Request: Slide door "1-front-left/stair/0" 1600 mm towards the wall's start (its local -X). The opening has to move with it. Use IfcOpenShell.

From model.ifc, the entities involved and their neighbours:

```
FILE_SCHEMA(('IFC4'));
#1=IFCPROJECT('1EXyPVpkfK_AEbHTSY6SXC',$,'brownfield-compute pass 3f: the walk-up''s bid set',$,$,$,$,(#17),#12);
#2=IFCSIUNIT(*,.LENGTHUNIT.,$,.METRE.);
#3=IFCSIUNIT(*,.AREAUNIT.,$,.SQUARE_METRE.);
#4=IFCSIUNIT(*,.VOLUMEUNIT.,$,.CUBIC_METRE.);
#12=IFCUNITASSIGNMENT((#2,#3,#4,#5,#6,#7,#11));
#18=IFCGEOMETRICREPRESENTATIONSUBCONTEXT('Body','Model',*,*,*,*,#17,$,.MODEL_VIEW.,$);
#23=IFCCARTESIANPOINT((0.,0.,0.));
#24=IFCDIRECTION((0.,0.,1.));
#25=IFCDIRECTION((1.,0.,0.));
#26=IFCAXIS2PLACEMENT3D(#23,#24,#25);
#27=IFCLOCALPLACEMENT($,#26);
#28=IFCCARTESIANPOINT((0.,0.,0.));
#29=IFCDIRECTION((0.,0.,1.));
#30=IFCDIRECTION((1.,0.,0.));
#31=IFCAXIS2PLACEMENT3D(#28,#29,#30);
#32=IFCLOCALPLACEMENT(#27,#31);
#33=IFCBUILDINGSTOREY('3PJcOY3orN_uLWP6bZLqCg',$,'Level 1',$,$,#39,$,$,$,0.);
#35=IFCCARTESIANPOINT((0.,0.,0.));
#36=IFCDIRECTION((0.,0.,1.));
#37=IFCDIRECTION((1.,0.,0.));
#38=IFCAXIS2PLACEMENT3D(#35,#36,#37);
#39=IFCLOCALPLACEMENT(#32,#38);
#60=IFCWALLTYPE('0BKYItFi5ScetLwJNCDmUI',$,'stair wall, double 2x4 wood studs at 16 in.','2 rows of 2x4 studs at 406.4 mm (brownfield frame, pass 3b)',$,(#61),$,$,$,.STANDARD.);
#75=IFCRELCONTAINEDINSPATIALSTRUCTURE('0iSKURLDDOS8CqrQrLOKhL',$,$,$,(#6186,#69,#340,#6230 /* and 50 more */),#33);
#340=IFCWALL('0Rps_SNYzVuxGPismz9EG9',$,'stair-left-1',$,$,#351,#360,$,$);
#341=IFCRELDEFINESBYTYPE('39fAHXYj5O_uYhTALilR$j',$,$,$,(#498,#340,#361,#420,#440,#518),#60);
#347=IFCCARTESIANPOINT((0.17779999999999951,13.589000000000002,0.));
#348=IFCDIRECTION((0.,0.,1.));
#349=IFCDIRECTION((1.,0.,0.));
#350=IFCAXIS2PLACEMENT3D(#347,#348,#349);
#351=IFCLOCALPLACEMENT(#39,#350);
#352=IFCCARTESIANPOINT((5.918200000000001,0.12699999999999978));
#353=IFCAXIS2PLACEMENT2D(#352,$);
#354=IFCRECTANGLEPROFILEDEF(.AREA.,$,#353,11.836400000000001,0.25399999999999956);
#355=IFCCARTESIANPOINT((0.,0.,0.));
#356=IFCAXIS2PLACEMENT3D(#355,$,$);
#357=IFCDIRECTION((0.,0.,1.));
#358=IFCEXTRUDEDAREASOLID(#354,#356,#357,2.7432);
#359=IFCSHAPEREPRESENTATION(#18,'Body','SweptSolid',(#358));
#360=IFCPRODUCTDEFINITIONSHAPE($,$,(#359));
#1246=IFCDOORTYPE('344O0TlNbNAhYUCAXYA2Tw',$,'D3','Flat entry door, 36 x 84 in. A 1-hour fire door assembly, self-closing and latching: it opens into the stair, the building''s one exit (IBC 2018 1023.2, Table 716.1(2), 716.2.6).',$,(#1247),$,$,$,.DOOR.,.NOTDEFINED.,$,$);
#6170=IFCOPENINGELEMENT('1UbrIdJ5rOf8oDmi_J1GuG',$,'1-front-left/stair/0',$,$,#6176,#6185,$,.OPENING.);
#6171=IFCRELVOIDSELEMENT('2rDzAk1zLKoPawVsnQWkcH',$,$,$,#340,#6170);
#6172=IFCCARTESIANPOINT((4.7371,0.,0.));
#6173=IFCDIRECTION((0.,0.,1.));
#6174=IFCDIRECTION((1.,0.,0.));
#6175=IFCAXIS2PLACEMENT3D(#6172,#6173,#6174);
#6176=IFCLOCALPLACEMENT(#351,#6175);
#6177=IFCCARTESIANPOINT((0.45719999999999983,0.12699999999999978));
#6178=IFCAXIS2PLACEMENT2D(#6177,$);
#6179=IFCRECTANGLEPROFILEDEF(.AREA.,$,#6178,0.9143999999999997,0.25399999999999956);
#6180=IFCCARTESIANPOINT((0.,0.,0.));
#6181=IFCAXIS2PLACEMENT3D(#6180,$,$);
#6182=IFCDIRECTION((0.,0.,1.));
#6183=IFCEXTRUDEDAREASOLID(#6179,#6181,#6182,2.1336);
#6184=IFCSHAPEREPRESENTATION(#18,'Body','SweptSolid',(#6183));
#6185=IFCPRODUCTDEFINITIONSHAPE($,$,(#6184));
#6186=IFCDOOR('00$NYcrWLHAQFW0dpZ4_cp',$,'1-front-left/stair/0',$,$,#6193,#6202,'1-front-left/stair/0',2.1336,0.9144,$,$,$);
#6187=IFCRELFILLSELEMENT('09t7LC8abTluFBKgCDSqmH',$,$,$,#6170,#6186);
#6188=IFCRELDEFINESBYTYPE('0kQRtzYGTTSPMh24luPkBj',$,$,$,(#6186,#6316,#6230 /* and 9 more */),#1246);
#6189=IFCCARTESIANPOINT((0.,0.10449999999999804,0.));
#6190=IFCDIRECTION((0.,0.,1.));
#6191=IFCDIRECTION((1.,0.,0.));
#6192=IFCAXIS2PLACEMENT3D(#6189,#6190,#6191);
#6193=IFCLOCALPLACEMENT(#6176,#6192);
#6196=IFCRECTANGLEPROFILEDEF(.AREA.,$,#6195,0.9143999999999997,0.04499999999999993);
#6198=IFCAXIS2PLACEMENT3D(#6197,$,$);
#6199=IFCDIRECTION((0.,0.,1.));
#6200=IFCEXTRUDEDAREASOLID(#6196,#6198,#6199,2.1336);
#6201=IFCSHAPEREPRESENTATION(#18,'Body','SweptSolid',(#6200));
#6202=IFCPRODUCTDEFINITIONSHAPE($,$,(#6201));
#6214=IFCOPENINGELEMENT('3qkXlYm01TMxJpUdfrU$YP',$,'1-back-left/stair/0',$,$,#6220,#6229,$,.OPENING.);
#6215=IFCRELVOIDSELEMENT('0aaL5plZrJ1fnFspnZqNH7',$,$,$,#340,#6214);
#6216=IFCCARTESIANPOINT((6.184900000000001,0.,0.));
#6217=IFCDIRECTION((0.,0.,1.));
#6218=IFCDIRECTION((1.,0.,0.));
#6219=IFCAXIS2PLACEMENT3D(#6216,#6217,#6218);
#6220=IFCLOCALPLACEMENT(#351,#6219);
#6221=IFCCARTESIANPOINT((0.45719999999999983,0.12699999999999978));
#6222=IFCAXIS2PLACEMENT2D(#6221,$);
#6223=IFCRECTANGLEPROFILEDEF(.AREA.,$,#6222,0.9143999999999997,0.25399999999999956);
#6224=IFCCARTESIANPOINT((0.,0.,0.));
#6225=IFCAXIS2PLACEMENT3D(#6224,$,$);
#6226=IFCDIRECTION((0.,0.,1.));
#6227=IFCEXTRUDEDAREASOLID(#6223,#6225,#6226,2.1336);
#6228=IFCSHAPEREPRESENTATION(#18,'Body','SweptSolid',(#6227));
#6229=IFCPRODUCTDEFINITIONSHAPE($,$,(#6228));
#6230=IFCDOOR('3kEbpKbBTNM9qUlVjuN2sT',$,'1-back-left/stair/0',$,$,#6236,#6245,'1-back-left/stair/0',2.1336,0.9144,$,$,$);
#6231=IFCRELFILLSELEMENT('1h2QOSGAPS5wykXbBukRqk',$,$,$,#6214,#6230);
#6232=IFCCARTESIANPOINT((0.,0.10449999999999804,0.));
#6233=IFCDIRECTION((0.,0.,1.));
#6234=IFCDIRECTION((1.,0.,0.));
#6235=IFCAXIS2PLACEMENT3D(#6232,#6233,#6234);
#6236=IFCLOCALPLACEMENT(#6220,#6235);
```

```python
import ifcopenshell
import ifcopenshell.api.geometry
import ifcopenshell.util.placement

model = ifcopenshell.open("model.ifc")

door = model.by_guid("00$NYcrWLHAQFW0dpZ4_cp")
opening = door.FillsVoids[0].RelatingOpeningElement
wall = opening.VoidsElements[0].RelatingBuildingElement

wall_matrix = ifcopenshell.util.placement.get_local_placement(wall.ObjectPlacement)
shift = wall_matrix[:3, 0] * -1.6
before = ifcopenshell.util.placement.get_local_placement(door.ObjectPlacement)[:3, 3].copy()

# The door is placed relative to its opening, so it follows when the opening moves.
matrix = ifcopenshell.util.placement.get_local_placement(opening.ObjectPlacement)
matrix[:3, 3] += shift
ifcopenshell.api.geometry.edit_object_placement(
    model, product=opening, matrix=matrix, is_si=False, should_transform_children=True
)

after = ifcopenshell.util.placement.get_local_placement(door.ObjectPlacement)[:3, 3]
print("door moved by", (after - before).round(3) + 0.0)

model.write("model_v2.ifc")
```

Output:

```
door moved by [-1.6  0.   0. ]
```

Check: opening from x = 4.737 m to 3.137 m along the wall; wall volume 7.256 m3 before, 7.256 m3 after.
